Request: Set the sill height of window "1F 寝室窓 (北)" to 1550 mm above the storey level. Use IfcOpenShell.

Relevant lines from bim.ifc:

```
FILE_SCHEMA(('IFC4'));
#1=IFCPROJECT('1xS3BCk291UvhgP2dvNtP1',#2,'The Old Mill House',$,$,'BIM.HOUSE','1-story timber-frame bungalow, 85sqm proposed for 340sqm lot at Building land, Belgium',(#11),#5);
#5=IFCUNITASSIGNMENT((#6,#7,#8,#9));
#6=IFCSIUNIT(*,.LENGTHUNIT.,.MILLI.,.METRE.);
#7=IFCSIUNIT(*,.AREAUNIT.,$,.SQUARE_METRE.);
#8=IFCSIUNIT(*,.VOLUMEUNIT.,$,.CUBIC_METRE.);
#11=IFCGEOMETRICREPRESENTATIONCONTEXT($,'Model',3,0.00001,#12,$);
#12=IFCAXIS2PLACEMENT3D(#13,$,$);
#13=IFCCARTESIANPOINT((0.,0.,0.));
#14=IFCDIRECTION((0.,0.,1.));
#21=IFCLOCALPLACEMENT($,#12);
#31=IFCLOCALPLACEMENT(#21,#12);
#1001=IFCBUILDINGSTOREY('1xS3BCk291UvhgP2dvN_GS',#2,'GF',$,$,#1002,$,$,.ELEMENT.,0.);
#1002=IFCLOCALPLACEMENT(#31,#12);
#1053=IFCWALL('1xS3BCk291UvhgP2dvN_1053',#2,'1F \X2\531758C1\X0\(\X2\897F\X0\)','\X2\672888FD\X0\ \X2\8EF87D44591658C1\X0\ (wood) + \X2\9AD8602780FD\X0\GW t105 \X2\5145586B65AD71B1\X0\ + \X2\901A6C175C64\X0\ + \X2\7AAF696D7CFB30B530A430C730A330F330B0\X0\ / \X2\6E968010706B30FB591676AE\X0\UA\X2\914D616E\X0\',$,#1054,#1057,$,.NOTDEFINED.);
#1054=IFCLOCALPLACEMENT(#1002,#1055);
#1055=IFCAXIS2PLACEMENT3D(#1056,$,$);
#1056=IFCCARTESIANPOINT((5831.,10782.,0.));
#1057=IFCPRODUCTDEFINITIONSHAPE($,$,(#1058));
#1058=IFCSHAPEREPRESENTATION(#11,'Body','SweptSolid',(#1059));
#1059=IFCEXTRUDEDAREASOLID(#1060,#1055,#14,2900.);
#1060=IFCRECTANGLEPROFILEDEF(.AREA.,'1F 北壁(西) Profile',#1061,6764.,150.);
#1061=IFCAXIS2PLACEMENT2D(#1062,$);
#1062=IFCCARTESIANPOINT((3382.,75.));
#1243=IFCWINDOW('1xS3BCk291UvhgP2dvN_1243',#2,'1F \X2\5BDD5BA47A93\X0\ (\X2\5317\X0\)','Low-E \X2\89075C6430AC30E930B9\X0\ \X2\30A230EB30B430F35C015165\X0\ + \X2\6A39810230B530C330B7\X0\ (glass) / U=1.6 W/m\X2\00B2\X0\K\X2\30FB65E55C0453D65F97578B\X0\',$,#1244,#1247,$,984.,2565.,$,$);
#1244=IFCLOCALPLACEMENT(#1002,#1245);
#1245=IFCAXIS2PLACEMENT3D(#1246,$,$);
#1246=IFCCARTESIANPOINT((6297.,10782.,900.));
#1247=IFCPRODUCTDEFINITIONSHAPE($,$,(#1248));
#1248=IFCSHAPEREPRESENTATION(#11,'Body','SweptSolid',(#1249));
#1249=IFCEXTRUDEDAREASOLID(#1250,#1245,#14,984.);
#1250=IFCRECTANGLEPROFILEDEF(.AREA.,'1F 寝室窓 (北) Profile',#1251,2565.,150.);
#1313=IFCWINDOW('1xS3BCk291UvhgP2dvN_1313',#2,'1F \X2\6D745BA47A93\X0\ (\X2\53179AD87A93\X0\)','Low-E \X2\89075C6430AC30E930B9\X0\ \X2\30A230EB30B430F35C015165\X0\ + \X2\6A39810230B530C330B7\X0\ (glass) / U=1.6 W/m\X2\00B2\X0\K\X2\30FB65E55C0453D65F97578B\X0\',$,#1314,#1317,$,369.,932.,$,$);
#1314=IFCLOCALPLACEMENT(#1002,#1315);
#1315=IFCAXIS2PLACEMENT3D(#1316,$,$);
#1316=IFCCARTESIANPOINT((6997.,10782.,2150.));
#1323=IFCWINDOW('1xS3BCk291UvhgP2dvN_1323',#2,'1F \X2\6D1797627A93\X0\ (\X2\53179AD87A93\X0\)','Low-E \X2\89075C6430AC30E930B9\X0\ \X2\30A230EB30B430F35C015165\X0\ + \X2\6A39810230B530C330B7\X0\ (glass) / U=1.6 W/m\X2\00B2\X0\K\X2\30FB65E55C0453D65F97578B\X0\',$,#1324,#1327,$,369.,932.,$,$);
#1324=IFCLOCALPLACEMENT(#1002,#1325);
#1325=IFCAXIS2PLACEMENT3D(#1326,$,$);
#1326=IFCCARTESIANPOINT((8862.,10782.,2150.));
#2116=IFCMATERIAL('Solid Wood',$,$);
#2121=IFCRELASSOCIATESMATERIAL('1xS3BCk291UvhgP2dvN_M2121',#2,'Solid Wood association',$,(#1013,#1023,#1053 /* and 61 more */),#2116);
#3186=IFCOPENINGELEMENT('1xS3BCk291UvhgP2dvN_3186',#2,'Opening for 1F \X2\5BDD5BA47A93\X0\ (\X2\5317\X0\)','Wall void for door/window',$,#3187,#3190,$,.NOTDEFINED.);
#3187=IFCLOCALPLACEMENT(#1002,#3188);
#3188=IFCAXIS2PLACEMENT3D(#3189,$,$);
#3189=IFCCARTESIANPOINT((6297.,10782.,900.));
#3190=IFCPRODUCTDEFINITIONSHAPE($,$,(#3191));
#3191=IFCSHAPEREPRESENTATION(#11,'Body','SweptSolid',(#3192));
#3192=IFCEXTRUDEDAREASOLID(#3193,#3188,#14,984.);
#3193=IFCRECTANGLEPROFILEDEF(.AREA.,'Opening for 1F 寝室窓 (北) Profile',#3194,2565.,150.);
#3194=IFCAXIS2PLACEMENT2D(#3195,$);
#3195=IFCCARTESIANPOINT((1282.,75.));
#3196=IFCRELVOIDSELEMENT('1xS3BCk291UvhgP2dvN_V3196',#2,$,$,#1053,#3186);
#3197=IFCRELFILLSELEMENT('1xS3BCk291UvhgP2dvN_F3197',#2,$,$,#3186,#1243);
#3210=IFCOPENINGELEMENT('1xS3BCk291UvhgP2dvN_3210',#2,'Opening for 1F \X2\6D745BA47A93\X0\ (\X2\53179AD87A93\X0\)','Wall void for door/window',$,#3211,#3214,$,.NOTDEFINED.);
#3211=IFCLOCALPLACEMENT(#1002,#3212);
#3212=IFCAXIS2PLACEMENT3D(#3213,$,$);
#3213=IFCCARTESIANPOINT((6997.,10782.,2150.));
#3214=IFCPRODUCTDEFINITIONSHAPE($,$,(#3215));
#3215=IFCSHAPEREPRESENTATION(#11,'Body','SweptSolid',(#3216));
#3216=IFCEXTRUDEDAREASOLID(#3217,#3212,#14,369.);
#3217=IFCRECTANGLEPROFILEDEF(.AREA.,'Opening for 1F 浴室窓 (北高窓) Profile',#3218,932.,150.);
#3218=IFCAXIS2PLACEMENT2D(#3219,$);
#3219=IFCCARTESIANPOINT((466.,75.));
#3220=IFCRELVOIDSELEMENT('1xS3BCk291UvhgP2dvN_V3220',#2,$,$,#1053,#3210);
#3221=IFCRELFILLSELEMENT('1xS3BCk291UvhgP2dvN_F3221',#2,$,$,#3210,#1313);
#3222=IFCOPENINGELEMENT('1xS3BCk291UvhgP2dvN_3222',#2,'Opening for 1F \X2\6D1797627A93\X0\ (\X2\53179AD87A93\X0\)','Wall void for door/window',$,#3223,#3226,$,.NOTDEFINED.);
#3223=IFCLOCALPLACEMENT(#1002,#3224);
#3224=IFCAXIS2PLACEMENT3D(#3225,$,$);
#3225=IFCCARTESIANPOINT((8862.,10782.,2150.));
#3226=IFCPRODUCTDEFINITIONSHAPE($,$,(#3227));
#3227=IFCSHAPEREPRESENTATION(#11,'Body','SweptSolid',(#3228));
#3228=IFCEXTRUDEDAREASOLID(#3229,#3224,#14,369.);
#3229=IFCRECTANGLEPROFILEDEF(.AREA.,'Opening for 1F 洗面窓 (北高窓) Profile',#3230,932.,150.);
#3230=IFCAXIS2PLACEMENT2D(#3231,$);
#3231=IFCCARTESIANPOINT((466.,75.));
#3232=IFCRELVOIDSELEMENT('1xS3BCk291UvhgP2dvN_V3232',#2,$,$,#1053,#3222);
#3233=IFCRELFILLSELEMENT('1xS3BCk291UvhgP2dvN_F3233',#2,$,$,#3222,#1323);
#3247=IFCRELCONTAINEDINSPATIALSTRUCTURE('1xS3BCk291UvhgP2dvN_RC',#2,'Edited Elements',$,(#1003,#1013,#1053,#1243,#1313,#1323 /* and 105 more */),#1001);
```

```python
import numpy as np
import ifcopenshell
import ifcopenshell.api.geometry
import ifcopenshell.geom
import ifcopenshell.util.element
import ifcopenshell.util.placement
import ifcopenshell.util.shape
import ifcopenshell.util.unit

model = ifcopenshell.open("bim.ifc")
unit_scale = ifcopenshell.util.unit.calculate_unit_scale(model)

window = model.by_guid("1xS3BCk291UvhgP2dvN_1243")
opening = window.FillsVoids[0].RelatingOpeningElement
storey = ifcopenshell.util.element.get_container(window, ifc_class="IfcBuildingStorey")
level = ifcopenshell.util.placement.get_local_placement(storey.ObjectPlacement)[2, 3]

# The opening's origin need not be at the sill, so measure its lowest point.
shape = ifcopenshell.geom.create_shape(ifcopenshell.geom.settings(), opening)
bottom = ifcopenshell.util.shape.get_shape_bottom_elevation(shape, shape.geometry) / unit_scale
dz = level + 1.55 / unit_scale - bottom

shift = np.array([0.0, 0.0, dz])
# The window is not placed relative to its opening, so move both.
for product in (opening, window):
    matrix = ifcopenshell.util.placement.get_local_placement(product.ObjectPlacement)
    matrix[:3, 3] += shift
    ifcopenshell.api.geometry.edit_object_placement(model, product=product, matrix=matrix, is_si=False)

print(f"moved by {dz * unit_scale:+.3f} m")

model.write("bim_updated.ifc")
```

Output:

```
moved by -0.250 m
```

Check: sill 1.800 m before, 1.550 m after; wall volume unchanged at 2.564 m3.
